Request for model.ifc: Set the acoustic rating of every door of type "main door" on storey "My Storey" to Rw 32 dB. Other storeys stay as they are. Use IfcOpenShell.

First a look at what the model holds.

```python
import ifcopenshell
import ifcopenshell.util.element

model = ifcopenshell.open("model.ifc")
print(model.schema)
storey = next(s for s in model.by_type("IfcBuildingStorey") if s.Name == "My Storey")
doors = [e for e in ifcopenshell.util.element.get_decomposition(storey) if e.is_a("IfcDoor")]
seen = {}
for e in doors:
    element_type = ifcopenshell.util.element.get_type(e)
    key = (element_type.Name if element_type != e and element_type else None, ifcopenshell.util.element.get_pset(e, "Pset_DoorCommon", "AcousticRating"))
    seen[key] = seen.get(key, 0) + 1
for (name, value), count in sorted(seen.items(), key=str):
    print(count, "x", name, "|", value)
```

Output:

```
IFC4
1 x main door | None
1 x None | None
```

```python
import ifcopenshell
import ifcopenshell.api.pset
import ifcopenshell.util.element

model = ifcopenshell.open("model.ifc")

storey = next(s for s in model.by_type("IfcBuildingStorey") if s.Name == "My Storey")
doors = [e for e in ifcopenshell.util.element.get_decomposition(storey) if e.is_a("IfcDoor")]

count = 0
for e in doors:
    element_type = ifcopenshell.util.element.get_type(e)
    if element_type in (None, e) or element_type.Name != "main door":
        continue
    # add_pset returns the element's existing set when there is one.
    pset = ifcopenshell.api.pset.add_pset(model, product=e, name="Pset_DoorCommon")
    ifcopenshell.api.pset.edit_pset(model, pset=pset, properties={"AcousticRating": "Rw 32 dB"})
    count += 1

print(count, "doors updated")

model.write("model_rev.ifc")
```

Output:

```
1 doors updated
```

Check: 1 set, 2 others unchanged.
